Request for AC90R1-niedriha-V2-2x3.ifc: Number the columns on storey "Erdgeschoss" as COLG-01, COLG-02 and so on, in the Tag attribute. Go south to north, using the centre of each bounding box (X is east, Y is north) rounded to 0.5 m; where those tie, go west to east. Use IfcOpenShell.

First a look at what the model holds.

```python
import ifcopenshell
import ifcopenshell.util.element
import ifcopenshell.util.placement

model = ifcopenshell.open("AC90R1-niedriha-V2-2x3.ifc")
print(model.schema)
storey = next(s for s in model.by_type("IfcBuildingStorey") if s.Name == "Erdgeschoss")
columns = [e for e in ifcopenshell.util.element.get_decomposition(storey) if e.is_a("IfcColumn")]
for e in sorted(columns, key=lambda e: e.id()):
    origin = ifcopenshell.util.placement.get_local_placement(e.ObjectPlacement)[:3, 3]
    print(e.id(), e.Tag, e.Name, origin.round(2) + 0.0, sep=" | ")
```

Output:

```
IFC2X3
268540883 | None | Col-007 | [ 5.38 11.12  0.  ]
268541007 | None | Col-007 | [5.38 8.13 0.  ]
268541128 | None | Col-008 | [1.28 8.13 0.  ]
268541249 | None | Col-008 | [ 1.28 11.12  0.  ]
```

```python
import ifcopenshell
import ifcopenshell.geom
import ifcopenshell.util.element
import ifcopenshell.util.shape

model = ifcopenshell.open("AC90R1-niedriha-V2-2x3.ifc")
settings = ifcopenshell.geom.settings()
settings.set("use-world-coords", True)


def centre(element):
    shape = ifcopenshell.geom.create_shape(settings, element)
    return ifcopenshell.util.shape.get_bbox_centroid(shape.geometry)


storey = next(s for s in model.by_type("IfcBuildingStorey") if s.Name == "Erdgeschoss")
columns = [e for e in ifcopenshell.util.element.get_decomposition(storey) if e.is_a("IfcColumn")]

# Insertion points can sit at a corner or the storey origin, so sort by the geometry (in metres).
centres = {e: centre(e) for e in columns}
columns.sort(key=lambda e: (round(centres[e][1] / 0.5), centres[e][0]))

for i, e in enumerate(columns, start=1):
    number = f"COLG-{i:02d}"
    e.Tag = number
    print(e.id(), number)

model.write("AC90R1-niedriha-V2-2x3_updated.ifc")
```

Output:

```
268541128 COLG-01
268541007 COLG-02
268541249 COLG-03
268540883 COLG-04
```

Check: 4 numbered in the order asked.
